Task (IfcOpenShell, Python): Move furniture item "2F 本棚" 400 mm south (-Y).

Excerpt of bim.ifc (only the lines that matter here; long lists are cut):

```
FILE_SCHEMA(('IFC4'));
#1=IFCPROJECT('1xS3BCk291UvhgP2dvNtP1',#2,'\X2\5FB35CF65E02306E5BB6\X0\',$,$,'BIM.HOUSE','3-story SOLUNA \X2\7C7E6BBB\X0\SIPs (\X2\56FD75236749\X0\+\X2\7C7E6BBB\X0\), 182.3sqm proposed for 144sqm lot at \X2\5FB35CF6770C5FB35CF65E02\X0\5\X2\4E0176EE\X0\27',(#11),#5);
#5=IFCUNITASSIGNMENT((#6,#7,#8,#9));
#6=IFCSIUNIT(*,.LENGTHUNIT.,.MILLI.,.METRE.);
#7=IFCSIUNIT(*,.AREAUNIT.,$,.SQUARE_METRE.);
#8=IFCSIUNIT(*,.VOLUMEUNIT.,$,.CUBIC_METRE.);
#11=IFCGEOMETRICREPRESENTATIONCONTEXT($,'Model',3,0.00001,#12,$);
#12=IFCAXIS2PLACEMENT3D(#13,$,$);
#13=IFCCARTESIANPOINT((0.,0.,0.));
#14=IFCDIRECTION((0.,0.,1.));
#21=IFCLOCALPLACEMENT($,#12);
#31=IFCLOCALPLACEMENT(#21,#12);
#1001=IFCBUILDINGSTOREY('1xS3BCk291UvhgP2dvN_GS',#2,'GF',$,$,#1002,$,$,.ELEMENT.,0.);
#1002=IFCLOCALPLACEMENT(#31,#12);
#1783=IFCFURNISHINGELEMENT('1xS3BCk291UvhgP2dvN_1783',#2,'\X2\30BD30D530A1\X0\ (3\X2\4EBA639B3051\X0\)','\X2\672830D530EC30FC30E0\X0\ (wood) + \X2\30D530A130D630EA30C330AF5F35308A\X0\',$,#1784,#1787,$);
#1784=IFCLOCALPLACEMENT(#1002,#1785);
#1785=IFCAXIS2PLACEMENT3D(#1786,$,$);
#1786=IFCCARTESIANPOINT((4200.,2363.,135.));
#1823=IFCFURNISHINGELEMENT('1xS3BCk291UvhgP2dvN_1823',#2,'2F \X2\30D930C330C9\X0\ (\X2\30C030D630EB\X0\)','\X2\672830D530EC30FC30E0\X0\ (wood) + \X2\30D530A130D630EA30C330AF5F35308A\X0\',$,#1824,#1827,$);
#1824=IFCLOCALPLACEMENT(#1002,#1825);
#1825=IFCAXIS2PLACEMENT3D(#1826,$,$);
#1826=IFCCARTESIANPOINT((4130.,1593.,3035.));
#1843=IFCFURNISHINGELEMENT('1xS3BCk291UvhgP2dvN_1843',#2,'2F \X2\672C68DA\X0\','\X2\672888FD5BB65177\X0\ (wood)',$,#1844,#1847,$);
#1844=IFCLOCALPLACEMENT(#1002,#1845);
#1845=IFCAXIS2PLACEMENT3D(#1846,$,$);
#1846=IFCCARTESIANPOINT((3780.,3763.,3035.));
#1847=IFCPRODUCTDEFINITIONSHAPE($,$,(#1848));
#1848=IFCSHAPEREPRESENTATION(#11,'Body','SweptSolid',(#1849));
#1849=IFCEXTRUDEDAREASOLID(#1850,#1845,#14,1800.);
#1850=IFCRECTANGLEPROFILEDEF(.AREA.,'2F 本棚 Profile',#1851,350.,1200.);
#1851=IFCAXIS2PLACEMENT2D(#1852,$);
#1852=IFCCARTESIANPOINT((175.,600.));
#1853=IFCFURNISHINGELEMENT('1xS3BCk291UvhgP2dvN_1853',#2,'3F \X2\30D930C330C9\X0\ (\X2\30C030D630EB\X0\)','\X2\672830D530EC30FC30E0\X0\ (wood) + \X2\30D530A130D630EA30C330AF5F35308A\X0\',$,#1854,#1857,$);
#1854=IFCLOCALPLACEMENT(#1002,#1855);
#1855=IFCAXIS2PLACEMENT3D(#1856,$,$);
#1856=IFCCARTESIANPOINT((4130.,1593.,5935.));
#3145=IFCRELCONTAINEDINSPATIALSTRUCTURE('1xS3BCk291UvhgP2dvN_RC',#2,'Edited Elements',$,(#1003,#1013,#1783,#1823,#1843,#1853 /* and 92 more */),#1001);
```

```python
import ifcopenshell
import ifcopenshell.api.geometry
import ifcopenshell.util.placement
import ifcopenshell.util.unit

model = ifcopenshell.open("bim.ifc")
unit_scale = ifcopenshell.util.unit.calculate_unit_scale(model)

item = model.by_id(1843)
matrix = ifcopenshell.util.placement.get_local_placement(item.ObjectPlacement)
matrix[1, 3] -= 0.4 / unit_scale
ifcopenshell.api.geometry.edit_object_placement(model, product=item, matrix=matrix, is_si=False)

print(ifcopenshell.util.placement.get_local_placement(item.ObjectPlacement).round(3) + 0.0)

model.write("bim_edited.ifc")
```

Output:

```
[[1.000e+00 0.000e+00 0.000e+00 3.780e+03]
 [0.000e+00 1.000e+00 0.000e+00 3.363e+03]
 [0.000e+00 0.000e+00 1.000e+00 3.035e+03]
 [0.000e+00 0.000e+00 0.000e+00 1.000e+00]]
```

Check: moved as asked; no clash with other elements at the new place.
